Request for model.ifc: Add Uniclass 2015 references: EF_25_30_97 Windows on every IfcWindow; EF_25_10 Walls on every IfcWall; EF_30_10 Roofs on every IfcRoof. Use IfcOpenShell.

First a look at what the model holds.

```python
import ifcopenshell

model = ifcopenshell.open("model.ifc")
print(model.schema)
print("classifications:", [c.Name for c in model.by_type("IfcClassification")])
for ifc_class in ("IfcDoor", "IfcRoof", "IfcStair", "IfcWall", "IfcWindow"):
    print(ifc_class, len(model.by_type(ifc_class)))
```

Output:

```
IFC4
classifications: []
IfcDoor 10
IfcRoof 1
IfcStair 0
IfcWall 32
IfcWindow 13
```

```python
import ifcopenshell
import ifcopenshell.api.classification

model = ifcopenshell.open("model.ifc")

system = ifcopenshell.api.classification.add_classification(model, classification="Uniclass 2015")

codes = {
    "IfcWindow": ("EF_25_30_97", "Windows"),
    "IfcWall": ("EF_25_10", "Walls"),
    "IfcRoof": ("EF_30_10", "Roofs"),
}
for ifc_class, (code, name) in codes.items():
    products = model.by_type(ifc_class)
    ifcopenshell.api.classification.add_reference(
        model, products=products, classification=system, identification=code, name=name
    )
    print(code, len(products))

model.write("model_updated.ifc")
```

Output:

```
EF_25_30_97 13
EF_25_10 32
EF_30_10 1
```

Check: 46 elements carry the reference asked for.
